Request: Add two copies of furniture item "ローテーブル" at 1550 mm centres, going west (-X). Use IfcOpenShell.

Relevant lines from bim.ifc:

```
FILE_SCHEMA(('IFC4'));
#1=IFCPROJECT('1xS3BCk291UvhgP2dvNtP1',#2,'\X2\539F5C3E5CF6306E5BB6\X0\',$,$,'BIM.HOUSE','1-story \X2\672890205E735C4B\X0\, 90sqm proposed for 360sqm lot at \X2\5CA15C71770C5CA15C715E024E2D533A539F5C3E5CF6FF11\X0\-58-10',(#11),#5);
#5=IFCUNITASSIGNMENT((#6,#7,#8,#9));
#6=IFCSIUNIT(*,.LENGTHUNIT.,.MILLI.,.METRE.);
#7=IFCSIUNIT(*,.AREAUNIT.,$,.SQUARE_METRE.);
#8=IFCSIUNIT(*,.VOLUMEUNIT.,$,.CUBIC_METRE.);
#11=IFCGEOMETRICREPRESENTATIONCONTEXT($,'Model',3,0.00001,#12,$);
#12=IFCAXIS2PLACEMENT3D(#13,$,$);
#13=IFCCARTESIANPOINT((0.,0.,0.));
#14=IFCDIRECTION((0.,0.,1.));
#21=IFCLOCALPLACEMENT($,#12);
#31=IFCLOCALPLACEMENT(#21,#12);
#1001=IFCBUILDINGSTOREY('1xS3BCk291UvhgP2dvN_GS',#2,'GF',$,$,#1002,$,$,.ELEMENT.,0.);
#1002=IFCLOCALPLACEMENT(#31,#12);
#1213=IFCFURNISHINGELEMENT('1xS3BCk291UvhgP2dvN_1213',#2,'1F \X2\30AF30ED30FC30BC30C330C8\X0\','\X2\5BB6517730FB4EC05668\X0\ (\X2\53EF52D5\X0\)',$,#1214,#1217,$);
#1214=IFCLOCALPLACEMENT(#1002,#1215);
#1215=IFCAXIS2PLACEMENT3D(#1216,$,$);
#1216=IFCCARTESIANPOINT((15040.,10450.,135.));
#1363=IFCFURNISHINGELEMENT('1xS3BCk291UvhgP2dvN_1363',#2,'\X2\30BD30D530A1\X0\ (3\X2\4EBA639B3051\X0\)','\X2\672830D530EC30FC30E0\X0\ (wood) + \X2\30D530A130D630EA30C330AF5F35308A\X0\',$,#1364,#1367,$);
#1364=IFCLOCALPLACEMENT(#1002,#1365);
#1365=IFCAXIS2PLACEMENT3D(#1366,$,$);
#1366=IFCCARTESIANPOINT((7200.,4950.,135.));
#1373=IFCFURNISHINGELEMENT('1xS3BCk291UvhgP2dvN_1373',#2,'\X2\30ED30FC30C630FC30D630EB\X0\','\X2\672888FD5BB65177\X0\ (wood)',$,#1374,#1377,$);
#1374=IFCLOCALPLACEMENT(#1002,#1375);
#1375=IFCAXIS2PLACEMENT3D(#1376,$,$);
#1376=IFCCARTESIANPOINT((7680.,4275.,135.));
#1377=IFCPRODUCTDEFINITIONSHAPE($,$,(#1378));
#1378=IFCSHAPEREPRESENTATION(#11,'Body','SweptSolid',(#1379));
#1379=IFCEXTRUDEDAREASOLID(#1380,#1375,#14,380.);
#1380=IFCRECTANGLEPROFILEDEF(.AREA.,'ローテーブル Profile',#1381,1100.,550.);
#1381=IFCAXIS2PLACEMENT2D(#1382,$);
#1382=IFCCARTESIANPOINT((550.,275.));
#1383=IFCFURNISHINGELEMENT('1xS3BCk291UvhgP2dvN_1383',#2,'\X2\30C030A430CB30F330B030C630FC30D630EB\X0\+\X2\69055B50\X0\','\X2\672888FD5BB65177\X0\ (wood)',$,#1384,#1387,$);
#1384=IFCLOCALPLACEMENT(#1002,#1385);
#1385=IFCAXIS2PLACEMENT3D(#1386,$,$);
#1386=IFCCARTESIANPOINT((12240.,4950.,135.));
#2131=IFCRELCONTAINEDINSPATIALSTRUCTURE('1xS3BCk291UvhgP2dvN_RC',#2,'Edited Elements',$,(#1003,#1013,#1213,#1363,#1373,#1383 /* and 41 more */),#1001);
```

```python
import numpy as np
import ifcopenshell
import ifcopenshell.api.geometry
import ifcopenshell.api.root
import ifcopenshell.util.element
import ifcopenshell.util.placement

model = ifcopenshell.open("bim.ifc")


def reuse_history(source, copy):
    """copy_class also copies each property set's owner history, people and application; keep the originals."""
    for rel in copy.IsDefinedBy:
        if rel.is_a("IfcRelDefinesByProperties") and (history := rel.RelatingPropertyDefinition.OwnerHistory):
            rel.RelatingPropertyDefinition.OwnerHistory = source.OwnerHistory
            ifcopenshell.util.element.remove_deep2(model, history)


source = model.by_guid("1xS3BCk291UvhgP2dvN_1373")
base = ifcopenshell.util.placement.get_local_placement(source.ObjectPlacement)
step = np.array([-1.0, 0.0, 0.0]) * 1550.0

for i in range(1, 3):
    copy = ifcopenshell.api.root.copy_class(model, product=source)
    copy.Representation = ifcopenshell.util.element.copy_deep(
        model, source.Representation, exclude=["IfcGeometricRepresentationContext", "IfcRepresentationMap"]
    )
    reuse_history(source, copy)
    matrix = base.copy()
    matrix[:3, 3] += i * step
    print("added at", matrix[:3, 3].round(3) + 0.0)
    ifcopenshell.api.geometry.edit_object_placement(model, product=copy, matrix=matrix, is_si=False)

model.write("bim_v2.ifc")
```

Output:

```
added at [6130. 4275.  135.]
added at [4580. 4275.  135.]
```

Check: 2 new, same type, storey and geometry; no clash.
